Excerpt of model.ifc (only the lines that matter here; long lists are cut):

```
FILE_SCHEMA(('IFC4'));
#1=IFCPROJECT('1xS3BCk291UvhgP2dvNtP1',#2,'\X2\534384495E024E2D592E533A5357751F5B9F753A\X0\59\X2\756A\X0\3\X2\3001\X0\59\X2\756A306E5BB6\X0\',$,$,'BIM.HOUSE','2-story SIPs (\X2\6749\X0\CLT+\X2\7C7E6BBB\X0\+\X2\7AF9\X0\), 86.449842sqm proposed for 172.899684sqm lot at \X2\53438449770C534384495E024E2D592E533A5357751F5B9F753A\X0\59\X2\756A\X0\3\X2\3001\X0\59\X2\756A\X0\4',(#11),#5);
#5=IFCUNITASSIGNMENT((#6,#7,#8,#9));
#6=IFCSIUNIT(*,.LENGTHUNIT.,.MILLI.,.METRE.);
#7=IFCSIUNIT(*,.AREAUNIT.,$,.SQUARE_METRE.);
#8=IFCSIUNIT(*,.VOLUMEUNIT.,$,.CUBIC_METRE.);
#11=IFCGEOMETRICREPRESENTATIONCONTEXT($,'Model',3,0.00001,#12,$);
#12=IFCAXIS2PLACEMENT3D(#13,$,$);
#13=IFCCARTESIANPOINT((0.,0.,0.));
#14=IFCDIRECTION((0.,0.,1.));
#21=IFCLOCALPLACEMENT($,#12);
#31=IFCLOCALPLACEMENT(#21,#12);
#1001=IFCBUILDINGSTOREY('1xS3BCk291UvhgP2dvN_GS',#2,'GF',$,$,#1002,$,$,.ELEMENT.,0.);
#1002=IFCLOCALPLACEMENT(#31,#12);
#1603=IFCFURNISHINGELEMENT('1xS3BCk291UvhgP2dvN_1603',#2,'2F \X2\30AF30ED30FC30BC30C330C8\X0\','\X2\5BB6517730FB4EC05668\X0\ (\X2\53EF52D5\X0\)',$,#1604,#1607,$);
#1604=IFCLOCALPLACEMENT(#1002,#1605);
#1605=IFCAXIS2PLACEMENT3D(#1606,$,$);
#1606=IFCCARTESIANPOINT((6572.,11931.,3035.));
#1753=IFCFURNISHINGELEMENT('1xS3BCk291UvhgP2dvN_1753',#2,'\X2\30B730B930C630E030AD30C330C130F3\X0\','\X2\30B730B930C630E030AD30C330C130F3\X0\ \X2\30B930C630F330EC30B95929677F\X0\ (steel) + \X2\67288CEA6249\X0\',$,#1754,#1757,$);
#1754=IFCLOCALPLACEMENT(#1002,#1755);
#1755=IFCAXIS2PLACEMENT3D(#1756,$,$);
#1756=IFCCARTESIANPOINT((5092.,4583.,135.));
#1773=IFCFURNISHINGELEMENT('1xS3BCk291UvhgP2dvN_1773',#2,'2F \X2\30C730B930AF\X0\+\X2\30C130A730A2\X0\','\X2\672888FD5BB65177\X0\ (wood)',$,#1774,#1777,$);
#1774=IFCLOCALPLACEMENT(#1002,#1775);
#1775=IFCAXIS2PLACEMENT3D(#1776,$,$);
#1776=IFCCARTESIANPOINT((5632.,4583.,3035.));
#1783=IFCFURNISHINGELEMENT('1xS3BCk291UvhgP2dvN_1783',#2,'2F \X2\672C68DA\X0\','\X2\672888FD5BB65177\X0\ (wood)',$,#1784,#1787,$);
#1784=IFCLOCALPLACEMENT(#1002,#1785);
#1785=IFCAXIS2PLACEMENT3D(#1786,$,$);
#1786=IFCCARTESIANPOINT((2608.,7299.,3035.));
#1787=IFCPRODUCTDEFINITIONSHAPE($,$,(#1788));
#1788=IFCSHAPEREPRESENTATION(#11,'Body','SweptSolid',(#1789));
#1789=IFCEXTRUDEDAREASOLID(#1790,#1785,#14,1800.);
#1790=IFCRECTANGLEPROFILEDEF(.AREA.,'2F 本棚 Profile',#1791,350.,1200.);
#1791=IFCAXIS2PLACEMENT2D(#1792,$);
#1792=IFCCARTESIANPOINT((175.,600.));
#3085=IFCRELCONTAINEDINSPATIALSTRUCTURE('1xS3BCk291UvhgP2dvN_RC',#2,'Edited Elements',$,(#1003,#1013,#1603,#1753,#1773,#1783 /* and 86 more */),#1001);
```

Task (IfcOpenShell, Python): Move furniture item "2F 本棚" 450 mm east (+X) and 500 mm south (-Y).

```python
import ifcopenshell
import ifcopenshell.api.geometry
import ifcopenshell.util.placement

model = ifcopenshell.open("model.ifc")

item = model.by_guid("1xS3BCk291UvhgP2dvN_1783")
matrix = ifcopenshell.util.placement.get_local_placement(item.ObjectPlacement)
matrix[0, 3] += 450.0
matrix[1, 3] -= 500.0
ifcopenshell.api.geometry.edit_object_placement(model, product=item, matrix=matrix, is_si=False)

print(ifcopenshell.util.placement.get_local_placement(item.ObjectPlacement).round(3) + 0.0)

model.write("model_edited.ifc")
```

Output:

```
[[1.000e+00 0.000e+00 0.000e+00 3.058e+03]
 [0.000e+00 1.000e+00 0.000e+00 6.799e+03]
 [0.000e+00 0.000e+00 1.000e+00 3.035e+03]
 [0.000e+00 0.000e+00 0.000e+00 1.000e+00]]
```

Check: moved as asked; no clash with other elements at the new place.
